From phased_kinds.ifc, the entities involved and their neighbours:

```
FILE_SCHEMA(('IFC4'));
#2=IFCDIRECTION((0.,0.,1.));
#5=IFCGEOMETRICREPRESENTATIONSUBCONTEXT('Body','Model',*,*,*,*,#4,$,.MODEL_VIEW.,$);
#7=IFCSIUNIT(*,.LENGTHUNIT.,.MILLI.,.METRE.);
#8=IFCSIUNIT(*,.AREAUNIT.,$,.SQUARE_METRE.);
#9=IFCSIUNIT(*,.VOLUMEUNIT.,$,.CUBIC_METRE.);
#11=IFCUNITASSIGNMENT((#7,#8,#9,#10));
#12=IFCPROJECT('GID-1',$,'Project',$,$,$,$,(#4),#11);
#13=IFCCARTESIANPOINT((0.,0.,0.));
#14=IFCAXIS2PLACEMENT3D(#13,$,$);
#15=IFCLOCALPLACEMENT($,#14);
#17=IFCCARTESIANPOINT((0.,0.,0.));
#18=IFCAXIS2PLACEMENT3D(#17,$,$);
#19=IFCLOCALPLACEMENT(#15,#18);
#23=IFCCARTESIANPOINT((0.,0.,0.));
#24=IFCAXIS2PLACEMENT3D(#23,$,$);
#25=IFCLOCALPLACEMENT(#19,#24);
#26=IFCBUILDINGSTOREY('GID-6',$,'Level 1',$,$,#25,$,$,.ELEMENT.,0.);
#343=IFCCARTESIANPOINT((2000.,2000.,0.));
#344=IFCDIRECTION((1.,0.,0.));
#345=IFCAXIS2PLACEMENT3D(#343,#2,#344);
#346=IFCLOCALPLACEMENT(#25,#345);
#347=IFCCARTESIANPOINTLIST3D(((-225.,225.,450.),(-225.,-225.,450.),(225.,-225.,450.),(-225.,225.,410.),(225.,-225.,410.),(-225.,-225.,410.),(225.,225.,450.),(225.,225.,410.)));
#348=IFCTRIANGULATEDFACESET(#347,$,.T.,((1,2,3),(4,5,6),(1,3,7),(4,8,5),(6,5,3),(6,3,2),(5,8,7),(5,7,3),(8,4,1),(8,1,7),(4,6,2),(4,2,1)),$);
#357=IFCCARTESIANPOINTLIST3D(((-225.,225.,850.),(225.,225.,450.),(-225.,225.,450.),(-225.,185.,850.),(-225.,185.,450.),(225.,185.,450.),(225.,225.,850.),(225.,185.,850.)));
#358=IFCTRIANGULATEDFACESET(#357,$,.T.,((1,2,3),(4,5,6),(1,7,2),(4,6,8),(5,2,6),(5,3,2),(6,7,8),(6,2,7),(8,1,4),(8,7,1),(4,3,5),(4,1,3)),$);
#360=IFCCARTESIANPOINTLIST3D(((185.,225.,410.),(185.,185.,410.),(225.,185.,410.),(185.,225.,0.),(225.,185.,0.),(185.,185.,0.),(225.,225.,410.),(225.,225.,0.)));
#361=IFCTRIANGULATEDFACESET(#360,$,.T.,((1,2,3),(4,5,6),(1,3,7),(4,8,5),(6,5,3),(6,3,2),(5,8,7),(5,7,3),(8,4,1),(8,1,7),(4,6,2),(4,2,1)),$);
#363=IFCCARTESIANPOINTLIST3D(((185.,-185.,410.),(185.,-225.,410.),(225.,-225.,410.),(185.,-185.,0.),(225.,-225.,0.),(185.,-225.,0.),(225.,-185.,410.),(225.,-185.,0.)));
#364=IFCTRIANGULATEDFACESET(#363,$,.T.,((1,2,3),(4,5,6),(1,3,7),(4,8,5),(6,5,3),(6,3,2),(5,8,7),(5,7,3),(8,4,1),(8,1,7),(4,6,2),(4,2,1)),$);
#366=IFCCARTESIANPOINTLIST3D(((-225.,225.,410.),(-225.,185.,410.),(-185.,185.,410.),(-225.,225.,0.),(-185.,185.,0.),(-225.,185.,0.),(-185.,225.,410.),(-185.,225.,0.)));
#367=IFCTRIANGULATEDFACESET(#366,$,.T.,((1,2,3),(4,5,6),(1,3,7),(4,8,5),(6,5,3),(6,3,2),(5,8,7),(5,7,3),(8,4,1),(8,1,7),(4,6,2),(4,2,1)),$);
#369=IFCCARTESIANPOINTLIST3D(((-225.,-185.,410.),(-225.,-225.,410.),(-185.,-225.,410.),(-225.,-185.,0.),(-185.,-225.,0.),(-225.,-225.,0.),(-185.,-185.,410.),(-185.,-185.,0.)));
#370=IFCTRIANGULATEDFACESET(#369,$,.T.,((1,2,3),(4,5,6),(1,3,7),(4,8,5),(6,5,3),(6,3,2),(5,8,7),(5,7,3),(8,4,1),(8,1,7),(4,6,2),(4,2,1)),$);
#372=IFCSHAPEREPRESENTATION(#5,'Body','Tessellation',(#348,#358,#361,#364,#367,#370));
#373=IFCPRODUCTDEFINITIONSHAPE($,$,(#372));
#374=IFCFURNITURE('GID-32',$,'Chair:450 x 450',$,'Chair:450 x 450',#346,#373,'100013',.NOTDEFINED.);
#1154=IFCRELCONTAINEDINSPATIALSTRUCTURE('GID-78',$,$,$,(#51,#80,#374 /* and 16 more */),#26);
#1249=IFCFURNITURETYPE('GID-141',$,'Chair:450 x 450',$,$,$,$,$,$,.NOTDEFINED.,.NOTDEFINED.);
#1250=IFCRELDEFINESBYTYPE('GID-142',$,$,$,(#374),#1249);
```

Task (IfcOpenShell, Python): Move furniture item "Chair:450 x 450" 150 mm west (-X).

```python
import ifcopenshell
import ifcopenshell.api.geometry
import ifcopenshell.util.placement
import ifcopenshell.util.unit

model = ifcopenshell.open("phased_kinds.ifc")
unit_scale = ifcopenshell.util.unit.calculate_unit_scale(model)

item = model.by_guid("GID-32")
matrix = ifcopenshell.util.placement.get_local_placement(item.ObjectPlacement)
matrix[0, 3] -= 0.15 / unit_scale
ifcopenshell.api.geometry.edit_object_placement(model, product=item, matrix=matrix, is_si=False)

print(ifcopenshell.util.placement.get_local_placement(item.ObjectPlacement).round(3) + 0.0)

model.write("phased_kinds_edited.ifc")
```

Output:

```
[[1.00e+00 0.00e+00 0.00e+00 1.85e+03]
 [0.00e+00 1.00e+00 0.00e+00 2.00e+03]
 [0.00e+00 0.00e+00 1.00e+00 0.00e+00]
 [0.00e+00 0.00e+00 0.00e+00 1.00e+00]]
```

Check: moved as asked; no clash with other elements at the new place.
